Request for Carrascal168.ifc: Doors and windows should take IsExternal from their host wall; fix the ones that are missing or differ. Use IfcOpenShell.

First a look at what the model holds.

```python
import ifcopenshell
import ifcopenshell.util.element

model = ifcopenshell.open("Carrascal168.ifc")
print(model.schema)
seen = {}
for e in model.by_type("IfcDoor") + model.by_type("IfcWindow"):
    if not e.FillsVoids:
        continue
    host = e.FillsVoids[0].RelatingOpeningElement.VoidsElements[0].RelatingBuildingElement
    own = ifcopenshell.util.element.get_pset(e, f"Pset_{e.is_a()[3:].removesuffix('StandardCase')}Common", "IsExternal")
    wall = ifcopenshell.util.element.get_pset(host, "Pset_WallCommon", "IsExternal")
    seen[e.is_a(), own, wall] = seen.get((e.is_a(), own, wall), 0) + 1
for (cls, own, wall), count in sorted(seen.items(), key=str):
    print(count, cls, "IsExternal:", own, "| host wall:", wall)
```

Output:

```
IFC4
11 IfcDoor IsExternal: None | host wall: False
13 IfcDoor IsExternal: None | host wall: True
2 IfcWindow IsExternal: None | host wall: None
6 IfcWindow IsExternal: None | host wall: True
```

```python
import ifcopenshell
import ifcopenshell.api.pset
import ifcopenshell.util.element

model = ifcopenshell.open("Carrascal168.ifc")

count = 0
for ifc_class, pset_name in (("IfcDoor", "Pset_DoorCommon"), ("IfcWindow", "Pset_WindowCommon")):
    for e in model.by_type(ifc_class):
        if not e.FillsVoids:
            continue
        host = e.FillsVoids[0].RelatingOpeningElement.VoidsElements[0].RelatingBuildingElement
        external = ifcopenshell.util.element.get_pset(host, "Pset_WallCommon", "IsExternal")
        if external is None or ifcopenshell.util.element.get_pset(e, pset_name, "IsExternal") == external:
            continue
        pset = ifcopenshell.api.pset.add_pset(model, product=e, name=pset_name)
        ifcopenshell.api.pset.edit_pset(model, pset=pset, properties={"IsExternal": external})
        count += 1

print(count, "updated")

model.write("Carrascal168_rev.ifc")
```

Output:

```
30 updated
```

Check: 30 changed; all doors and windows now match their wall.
